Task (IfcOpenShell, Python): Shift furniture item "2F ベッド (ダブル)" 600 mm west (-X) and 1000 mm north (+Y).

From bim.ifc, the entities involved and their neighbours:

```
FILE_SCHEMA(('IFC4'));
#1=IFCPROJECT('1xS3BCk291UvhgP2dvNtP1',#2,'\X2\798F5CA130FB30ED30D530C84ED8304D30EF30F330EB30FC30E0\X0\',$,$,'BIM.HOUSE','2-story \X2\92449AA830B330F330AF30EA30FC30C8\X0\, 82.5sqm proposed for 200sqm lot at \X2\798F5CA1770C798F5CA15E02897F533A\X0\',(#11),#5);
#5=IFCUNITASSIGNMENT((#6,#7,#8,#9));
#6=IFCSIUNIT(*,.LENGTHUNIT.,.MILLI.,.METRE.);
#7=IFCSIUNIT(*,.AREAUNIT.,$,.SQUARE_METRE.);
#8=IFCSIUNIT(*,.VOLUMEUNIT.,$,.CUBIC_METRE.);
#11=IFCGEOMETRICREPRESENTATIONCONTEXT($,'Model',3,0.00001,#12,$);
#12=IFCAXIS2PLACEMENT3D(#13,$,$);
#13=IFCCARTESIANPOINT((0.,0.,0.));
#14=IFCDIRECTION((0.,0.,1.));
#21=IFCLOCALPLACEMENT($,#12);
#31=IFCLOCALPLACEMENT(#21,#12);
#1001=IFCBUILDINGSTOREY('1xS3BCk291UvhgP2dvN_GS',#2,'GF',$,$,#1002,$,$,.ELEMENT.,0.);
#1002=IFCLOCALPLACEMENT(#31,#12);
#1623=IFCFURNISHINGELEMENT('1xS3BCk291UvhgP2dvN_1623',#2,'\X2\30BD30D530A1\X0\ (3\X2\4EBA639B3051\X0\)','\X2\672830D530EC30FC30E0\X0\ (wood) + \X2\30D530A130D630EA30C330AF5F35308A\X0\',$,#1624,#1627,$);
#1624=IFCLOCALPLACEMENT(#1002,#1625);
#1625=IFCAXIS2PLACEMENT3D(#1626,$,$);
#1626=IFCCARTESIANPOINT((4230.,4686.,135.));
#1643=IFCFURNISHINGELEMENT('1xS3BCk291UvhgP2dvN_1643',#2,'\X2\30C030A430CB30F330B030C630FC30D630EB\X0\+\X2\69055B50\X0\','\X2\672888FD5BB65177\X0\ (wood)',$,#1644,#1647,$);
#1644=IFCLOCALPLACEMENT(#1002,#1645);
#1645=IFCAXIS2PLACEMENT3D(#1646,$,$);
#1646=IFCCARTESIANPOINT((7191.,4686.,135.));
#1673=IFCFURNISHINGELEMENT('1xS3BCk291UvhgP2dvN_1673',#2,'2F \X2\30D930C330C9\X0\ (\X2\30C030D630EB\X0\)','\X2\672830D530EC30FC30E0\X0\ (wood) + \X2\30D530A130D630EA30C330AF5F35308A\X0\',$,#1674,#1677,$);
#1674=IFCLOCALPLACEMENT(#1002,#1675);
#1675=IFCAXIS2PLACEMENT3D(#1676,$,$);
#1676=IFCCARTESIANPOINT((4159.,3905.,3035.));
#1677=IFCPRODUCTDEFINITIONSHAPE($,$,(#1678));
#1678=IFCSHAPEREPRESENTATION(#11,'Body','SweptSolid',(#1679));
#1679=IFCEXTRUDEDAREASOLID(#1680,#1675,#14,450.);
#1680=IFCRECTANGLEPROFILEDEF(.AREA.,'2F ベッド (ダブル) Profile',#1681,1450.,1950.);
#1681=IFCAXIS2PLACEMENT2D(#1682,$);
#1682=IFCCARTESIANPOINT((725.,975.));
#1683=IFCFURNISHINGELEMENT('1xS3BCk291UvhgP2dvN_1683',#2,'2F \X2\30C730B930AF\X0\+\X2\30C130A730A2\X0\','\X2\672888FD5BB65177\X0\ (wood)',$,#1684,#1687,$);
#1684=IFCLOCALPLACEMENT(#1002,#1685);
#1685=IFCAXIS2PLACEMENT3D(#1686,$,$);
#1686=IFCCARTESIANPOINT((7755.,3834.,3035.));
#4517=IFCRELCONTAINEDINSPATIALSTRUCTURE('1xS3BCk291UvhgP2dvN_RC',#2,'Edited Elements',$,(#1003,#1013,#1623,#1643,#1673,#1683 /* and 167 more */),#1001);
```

```python
import ifcopenshell
import ifcopenshell.api.geometry
import ifcopenshell.util.placement
import ifcopenshell.util.unit

model = ifcopenshell.open("bim.ifc")
unit_scale = ifcopenshell.util.unit.calculate_unit_scale(model)

item = model.by_guid("1xS3BCk291UvhgP2dvN_1673")
matrix = ifcopenshell.util.placement.get_local_placement(item.ObjectPlacement)
matrix[0, 3] -= 0.6 / unit_scale
matrix[1, 3] += 1 / unit_scale
ifcopenshell.api.geometry.edit_object_placement(model, product=item, matrix=matrix, is_si=False)

print(ifcopenshell.util.placement.get_local_placement(item.ObjectPlacement).round(3) + 0.0)

model.write("bim_rev.ifc")
```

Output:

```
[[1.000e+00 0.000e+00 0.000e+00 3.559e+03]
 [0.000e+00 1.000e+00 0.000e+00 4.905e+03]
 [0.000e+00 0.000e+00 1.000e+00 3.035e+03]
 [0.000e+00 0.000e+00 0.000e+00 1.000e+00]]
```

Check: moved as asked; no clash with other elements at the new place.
